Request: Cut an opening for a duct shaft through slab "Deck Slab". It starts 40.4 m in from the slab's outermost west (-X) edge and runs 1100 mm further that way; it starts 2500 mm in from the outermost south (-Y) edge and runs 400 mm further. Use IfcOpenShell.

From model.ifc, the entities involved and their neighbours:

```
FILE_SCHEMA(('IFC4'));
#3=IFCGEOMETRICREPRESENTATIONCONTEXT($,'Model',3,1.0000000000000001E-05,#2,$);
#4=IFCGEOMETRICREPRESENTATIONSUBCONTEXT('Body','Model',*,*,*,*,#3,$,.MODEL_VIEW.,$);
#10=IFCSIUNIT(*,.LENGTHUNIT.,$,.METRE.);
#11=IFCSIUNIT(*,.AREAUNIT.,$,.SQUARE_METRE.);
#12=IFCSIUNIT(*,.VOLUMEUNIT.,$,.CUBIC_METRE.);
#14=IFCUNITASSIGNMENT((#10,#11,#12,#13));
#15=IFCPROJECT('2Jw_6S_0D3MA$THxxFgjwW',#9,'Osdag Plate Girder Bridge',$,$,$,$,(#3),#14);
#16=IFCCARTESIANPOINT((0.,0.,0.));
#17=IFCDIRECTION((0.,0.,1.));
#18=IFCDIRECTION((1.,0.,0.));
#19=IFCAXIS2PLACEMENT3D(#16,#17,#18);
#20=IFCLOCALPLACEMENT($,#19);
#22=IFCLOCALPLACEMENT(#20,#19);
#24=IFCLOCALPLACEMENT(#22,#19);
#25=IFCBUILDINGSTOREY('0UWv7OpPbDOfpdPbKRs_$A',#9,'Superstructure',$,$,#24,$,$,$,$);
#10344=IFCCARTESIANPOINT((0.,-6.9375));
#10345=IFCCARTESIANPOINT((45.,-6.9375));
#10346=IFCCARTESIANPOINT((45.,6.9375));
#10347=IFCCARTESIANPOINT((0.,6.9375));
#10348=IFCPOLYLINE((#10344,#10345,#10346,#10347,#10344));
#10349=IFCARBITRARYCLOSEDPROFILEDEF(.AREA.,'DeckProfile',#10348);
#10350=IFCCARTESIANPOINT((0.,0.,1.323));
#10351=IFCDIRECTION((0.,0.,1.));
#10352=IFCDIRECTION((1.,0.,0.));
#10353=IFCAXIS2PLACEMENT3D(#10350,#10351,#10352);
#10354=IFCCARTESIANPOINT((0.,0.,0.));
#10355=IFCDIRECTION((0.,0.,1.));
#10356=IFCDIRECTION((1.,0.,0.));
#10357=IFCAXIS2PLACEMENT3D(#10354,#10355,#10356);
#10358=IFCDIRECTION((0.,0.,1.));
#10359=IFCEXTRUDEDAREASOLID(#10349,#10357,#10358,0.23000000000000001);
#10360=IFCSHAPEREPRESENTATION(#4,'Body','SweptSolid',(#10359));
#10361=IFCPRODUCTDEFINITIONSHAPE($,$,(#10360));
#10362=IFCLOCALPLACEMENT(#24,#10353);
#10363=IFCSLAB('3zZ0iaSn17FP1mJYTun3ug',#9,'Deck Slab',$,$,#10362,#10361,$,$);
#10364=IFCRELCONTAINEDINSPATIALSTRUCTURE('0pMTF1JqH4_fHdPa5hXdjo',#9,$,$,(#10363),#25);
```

```python
import numpy as np
import ifcopenshell
import ifcopenshell.api.feature
import ifcopenshell.api.geometry
import ifcopenshell.api.root
import ifcopenshell.geom
import ifcopenshell.util.placement
import ifcopenshell.util.representation
import ifcopenshell.util.shape
import ifcopenshell.util.unit

model = ifcopenshell.open("model.ifc")
unit_scale = ifcopenshell.util.unit.calculate_unit_scale(model)
settings = ifcopenshell.geom.settings()


def volume(element):
    """Net volume in cubic metres, openings subtracted."""
    shape = ifcopenshell.geom.create_shape(settings, element)
    return ifcopenshell.util.shape.get_volume(shape.geometry)


slab = model.by_guid("3zZ0iaSn17FP1mJYTun3ug")
before = volume(slab)

# Extent in the slab's own axes, in metres. The edges named are its -X and -Y sides.
slab_shape = ifcopenshell.geom.create_shape(settings, slab)
vertices = ifcopenshell.util.shape.get_vertices(slab_shape.geometry)
x_min, y_min, bottom = vertices.min(axis=0)
top = vertices[:, 2].max()

opening = ifcopenshell.api.root.create_entity(model, ifc_class="IfcOpeningElement", name="Duct shaft opening", predefined_type="OPENING")
context = ifcopenshell.util.representation.get_context(model, "Model", "Body", "MODEL_VIEW")
width, depth = 1.1, 0.4
outline = [(0.0, 0.0), (width, 0.0), (width, depth), (0.0, depth), (0.0, 0.0)]
# Overshoot both faces by 50 mm so the cut is clean.
shape = ifcopenshell.api.geometry.add_slab_representation(
    model, context=context, depth=top - bottom + 0.1, polyline=outline
)
ifcopenshell.api.geometry.assign_representation(model, product=opening, representation=shape)

matrix = ifcopenshell.util.placement.get_local_placement(slab.ObjectPlacement)
matrix[:, 3] = matrix @ np.append(np.array([x_min + 40.4, y_min + 2.5, bottom - 0.05]) / unit_scale, 1.0)
ifcopenshell.api.geometry.edit_object_placement(model, product=opening, matrix=matrix, is_si=False)
ifcopenshell.api.feature.add_feature(model, feature=opening, element=slab)

after = volume(slab)

print(f"slab volume {before:.3f} -> {after:.3f} m3")

model.write("model-out.ifc")
```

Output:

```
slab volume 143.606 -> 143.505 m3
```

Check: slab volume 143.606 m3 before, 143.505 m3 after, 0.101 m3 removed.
